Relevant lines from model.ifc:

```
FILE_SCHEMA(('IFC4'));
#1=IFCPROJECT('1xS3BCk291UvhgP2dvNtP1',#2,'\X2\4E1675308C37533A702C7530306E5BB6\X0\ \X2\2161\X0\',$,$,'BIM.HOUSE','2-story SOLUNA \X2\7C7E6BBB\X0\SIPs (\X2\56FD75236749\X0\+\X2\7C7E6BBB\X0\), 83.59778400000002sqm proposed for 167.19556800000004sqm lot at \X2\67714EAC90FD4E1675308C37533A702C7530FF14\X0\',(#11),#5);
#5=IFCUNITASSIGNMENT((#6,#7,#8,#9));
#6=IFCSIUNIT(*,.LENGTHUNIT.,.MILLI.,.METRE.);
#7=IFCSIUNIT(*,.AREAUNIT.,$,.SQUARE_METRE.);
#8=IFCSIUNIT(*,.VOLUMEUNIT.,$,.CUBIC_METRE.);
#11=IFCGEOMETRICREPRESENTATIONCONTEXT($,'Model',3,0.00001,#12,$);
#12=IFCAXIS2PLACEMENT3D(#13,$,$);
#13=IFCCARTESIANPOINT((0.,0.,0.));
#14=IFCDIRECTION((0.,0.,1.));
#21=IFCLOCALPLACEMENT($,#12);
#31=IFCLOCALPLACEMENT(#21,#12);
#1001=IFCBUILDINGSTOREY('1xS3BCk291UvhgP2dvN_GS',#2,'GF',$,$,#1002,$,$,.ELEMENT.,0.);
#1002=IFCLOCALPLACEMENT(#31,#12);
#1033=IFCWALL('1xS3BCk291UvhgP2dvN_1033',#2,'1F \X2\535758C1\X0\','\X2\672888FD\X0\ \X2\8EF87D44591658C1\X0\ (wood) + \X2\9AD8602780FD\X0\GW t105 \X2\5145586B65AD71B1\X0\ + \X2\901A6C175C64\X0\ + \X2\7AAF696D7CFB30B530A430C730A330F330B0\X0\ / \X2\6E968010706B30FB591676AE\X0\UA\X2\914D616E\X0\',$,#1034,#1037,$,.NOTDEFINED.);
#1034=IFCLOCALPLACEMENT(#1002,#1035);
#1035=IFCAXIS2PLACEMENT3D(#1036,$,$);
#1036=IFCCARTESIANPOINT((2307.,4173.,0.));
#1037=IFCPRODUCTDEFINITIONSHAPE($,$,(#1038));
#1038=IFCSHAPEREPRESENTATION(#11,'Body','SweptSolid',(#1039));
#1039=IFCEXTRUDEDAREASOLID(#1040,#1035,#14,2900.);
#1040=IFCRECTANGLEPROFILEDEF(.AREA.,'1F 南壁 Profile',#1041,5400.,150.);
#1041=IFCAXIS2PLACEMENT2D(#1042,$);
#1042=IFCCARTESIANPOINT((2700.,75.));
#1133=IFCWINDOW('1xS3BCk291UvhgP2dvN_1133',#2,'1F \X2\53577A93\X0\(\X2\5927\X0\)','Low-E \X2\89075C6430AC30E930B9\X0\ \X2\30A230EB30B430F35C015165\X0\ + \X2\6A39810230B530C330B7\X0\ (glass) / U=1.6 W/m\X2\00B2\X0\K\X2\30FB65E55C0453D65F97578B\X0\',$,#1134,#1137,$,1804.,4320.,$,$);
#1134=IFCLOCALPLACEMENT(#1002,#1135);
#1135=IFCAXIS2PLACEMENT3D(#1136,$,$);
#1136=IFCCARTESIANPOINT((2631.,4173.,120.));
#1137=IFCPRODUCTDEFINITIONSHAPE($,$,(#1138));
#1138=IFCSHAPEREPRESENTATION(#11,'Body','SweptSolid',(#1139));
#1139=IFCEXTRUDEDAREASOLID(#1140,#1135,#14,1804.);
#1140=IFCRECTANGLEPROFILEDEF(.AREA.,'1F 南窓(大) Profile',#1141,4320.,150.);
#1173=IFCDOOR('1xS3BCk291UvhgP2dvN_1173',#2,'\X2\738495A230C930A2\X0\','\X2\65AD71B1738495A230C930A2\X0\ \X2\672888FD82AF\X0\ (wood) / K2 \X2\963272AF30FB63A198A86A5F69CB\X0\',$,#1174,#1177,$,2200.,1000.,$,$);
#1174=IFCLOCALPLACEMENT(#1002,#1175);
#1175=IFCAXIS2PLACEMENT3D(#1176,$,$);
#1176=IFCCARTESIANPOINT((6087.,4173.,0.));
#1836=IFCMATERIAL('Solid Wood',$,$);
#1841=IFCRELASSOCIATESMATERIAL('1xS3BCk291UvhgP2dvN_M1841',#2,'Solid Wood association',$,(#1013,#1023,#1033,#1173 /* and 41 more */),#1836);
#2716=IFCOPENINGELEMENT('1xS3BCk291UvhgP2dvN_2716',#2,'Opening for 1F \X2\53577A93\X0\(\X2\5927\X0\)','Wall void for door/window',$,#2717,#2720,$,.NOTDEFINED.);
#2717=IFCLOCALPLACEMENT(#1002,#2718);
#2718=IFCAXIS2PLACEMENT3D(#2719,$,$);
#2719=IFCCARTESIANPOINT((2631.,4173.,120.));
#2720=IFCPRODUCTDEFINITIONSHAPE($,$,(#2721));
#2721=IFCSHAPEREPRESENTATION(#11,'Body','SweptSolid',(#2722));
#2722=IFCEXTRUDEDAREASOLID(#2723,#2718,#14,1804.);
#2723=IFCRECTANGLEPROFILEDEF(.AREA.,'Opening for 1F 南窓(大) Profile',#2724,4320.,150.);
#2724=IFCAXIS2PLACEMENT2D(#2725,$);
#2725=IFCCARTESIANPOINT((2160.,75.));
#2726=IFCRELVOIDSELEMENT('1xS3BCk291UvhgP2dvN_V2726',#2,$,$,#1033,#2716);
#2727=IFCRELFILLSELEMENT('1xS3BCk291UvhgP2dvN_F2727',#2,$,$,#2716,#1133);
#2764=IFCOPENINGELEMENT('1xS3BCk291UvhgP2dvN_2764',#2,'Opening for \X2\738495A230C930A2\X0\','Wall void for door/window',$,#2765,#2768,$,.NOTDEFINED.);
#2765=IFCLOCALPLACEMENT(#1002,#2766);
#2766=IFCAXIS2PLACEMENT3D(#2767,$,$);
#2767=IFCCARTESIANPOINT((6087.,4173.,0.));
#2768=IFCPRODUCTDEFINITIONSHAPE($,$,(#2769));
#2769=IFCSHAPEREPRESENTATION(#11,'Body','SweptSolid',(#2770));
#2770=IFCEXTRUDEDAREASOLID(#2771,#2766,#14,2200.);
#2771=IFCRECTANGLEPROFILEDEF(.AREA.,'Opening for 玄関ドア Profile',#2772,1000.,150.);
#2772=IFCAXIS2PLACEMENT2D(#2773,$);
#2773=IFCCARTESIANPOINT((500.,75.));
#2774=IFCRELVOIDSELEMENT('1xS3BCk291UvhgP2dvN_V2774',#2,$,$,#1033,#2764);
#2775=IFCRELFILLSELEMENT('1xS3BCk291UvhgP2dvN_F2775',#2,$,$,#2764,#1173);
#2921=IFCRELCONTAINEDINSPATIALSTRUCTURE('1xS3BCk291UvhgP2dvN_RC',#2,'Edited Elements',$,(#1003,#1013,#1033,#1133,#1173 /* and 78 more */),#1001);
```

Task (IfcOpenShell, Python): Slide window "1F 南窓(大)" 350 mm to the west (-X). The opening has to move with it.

```python
import ifcopenshell
import ifcopenshell.api.geometry
import ifcopenshell.util.placement
import ifcopenshell.util.unit

model = ifcopenshell.open("model.ifc")
unit_scale = ifcopenshell.util.unit.calculate_unit_scale(model)

window = model.by_guid("1xS3BCk291UvhgP2dvN_1133")
opening = window.FillsVoids[0].RelatingOpeningElement
wall = opening.VoidsElements[0].RelatingBuildingElement

wall_matrix = ifcopenshell.util.placement.get_local_placement(wall.ObjectPlacement)
shift = wall_matrix[:3, 0] * -0.35 / unit_scale
before = ifcopenshell.util.placement.get_local_placement(window.ObjectPlacement)[:3, 3].copy()

# The window is not placed relative to its opening, so move both.
for product in (opening, window):
    matrix = ifcopenshell.util.placement.get_local_placement(product.ObjectPlacement)
    matrix[:3, 3] += shift
    ifcopenshell.api.geometry.edit_object_placement(model, product=product, matrix=matrix, is_si=False)

after = ifcopenshell.util.placement.get_local_placement(window.ObjectPlacement)[:3, 3]
print("window moved by", (after - before).round(3) + 0.0)

model.write("model_rev.ifc")
```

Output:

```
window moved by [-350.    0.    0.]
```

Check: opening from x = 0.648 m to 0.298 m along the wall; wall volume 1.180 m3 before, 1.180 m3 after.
